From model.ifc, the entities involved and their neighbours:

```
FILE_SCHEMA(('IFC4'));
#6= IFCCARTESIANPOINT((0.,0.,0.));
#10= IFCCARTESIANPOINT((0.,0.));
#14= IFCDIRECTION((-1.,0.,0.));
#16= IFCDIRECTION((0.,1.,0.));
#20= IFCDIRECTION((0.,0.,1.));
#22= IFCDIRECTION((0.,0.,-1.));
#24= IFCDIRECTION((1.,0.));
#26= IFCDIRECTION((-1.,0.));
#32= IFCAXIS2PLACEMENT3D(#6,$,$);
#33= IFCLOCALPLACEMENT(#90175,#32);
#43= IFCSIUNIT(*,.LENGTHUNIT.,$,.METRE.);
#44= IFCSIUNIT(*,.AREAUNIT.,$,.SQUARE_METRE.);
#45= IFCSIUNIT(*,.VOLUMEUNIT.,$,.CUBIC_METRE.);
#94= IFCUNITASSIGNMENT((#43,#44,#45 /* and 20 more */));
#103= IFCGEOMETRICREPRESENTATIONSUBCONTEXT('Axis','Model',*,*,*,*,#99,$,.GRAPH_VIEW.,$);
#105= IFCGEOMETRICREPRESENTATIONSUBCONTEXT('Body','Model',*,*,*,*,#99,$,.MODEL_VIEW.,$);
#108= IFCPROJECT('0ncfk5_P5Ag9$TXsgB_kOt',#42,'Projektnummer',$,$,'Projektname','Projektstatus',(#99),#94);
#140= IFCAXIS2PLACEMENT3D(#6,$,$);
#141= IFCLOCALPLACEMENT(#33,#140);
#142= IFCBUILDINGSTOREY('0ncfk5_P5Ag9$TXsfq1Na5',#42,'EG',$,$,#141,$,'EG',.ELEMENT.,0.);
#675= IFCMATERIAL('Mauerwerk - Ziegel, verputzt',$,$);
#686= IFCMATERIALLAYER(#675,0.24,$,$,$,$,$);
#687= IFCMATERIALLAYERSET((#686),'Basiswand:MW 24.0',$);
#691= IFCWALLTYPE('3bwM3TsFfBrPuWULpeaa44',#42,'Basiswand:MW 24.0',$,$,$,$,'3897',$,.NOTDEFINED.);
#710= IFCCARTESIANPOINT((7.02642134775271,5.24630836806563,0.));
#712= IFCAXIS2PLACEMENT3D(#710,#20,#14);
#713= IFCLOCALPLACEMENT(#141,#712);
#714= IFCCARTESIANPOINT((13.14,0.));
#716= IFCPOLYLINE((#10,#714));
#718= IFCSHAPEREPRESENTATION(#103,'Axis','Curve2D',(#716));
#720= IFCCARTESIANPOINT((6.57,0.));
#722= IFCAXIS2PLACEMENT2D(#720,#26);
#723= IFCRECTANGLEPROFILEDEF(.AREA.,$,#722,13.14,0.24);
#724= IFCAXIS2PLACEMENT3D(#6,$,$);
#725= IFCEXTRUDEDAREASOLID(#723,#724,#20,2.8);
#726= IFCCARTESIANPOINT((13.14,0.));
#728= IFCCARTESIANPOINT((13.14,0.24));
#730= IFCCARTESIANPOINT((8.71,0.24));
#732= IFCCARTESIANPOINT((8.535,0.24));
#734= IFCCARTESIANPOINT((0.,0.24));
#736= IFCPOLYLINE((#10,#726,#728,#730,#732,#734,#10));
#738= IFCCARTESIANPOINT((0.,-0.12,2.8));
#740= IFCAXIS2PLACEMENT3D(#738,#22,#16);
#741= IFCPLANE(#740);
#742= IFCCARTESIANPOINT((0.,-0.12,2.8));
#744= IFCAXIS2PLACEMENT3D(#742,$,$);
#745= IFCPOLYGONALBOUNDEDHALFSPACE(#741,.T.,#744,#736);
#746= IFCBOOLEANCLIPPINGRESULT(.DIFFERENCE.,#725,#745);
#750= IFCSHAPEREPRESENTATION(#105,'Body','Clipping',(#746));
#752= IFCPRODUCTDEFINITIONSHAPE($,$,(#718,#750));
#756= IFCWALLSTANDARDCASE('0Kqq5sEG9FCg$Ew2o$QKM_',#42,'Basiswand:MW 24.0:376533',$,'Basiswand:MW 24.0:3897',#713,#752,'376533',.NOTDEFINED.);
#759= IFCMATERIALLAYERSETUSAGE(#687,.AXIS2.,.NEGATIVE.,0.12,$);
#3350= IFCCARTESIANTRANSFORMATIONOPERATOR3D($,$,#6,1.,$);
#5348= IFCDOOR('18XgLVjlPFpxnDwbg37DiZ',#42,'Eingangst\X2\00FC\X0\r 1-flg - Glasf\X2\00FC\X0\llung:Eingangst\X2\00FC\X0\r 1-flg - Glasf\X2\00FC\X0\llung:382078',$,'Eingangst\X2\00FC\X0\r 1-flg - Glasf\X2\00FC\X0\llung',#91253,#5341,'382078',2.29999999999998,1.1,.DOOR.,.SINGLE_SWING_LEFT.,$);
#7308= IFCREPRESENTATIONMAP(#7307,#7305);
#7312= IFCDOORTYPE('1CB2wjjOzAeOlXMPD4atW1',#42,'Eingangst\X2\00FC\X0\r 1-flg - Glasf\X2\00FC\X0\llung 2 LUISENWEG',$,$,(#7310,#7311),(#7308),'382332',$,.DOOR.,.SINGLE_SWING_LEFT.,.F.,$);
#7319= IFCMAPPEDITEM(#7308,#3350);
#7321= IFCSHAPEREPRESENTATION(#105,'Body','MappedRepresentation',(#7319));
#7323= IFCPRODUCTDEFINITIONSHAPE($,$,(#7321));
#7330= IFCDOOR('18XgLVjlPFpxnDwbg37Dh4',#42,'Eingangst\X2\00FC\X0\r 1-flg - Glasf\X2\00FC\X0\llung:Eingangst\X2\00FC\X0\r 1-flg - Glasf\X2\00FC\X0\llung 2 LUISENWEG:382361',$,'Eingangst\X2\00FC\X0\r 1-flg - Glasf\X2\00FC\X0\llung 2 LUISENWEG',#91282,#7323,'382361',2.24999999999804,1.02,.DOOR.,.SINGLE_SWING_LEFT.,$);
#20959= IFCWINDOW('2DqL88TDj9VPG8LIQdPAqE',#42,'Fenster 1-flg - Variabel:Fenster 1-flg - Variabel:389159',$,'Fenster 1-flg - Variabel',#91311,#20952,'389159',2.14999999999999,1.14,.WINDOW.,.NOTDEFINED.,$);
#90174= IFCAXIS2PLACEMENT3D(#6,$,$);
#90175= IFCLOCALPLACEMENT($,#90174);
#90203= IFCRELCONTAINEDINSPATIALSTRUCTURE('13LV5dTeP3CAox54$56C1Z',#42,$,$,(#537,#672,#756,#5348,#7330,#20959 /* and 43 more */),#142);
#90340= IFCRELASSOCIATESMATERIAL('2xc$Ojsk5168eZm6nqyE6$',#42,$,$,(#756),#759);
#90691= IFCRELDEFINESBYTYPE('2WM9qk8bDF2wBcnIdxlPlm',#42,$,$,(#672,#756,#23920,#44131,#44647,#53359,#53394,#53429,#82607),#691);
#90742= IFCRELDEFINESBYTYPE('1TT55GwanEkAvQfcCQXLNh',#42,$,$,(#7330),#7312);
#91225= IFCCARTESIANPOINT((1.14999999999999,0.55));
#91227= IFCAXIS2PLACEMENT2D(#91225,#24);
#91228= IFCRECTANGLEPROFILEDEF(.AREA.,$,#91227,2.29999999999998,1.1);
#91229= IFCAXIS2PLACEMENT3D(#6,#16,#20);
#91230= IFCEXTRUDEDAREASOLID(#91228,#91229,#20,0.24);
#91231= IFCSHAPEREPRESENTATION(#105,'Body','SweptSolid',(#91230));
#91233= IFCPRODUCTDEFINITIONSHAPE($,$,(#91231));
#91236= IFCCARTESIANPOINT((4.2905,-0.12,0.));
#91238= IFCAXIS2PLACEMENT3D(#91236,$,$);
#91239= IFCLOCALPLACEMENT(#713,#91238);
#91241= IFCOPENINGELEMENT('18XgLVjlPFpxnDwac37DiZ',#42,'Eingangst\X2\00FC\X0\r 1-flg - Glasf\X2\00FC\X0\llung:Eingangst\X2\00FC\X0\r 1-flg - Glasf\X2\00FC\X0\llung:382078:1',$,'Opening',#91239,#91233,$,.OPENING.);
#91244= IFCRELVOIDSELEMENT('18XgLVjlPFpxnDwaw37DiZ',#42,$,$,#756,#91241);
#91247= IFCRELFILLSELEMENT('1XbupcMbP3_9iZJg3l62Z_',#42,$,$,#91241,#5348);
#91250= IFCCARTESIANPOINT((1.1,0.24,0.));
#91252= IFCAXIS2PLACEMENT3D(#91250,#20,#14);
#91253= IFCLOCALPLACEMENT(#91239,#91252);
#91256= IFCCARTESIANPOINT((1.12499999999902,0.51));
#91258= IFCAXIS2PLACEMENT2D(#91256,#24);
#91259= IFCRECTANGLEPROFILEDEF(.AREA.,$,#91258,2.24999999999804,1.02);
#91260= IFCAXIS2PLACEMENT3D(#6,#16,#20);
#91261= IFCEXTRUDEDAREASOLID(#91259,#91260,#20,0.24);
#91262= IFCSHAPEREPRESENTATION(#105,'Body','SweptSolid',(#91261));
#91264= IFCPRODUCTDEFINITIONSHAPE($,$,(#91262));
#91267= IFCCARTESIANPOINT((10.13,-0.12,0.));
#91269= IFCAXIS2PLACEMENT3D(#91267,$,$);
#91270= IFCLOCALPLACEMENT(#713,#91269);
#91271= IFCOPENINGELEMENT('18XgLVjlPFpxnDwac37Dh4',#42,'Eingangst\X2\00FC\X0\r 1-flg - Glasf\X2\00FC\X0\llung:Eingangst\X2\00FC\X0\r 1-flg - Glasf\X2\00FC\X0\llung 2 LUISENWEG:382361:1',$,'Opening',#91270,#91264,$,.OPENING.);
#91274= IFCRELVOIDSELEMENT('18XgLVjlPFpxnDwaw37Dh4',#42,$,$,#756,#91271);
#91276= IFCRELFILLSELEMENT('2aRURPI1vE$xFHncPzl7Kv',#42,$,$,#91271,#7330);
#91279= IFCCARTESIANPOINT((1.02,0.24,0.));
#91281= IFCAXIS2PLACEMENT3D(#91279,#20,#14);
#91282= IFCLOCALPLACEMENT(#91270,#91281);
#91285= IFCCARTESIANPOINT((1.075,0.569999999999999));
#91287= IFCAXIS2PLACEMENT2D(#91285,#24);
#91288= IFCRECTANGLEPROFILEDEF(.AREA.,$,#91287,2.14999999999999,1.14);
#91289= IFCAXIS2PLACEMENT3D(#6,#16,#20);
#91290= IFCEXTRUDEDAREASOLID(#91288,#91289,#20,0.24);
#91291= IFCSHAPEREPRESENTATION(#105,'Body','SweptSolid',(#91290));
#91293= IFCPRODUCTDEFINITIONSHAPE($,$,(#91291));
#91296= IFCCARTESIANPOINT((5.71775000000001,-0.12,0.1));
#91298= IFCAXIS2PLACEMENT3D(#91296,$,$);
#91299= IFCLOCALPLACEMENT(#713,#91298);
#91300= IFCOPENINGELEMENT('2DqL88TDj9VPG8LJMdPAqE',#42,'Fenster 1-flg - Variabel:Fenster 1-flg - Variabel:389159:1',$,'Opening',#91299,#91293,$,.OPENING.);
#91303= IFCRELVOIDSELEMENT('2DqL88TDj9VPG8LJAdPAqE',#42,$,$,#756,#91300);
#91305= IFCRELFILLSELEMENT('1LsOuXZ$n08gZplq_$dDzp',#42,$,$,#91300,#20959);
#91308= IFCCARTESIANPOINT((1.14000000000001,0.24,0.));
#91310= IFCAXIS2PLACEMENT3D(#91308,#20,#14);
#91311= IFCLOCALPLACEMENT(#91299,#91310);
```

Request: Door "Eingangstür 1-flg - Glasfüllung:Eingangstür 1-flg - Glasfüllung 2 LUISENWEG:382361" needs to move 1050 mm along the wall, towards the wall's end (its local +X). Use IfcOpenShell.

```python
import ifcopenshell
import ifcopenshell.api.geometry
import ifcopenshell.util.placement

model = ifcopenshell.open("model.ifc")

door = model.by_guid("18XgLVjlPFpxnDwbg37Dh4")
opening = door.FillsVoids[0].RelatingOpeningElement
wall = opening.VoidsElements[0].RelatingBuildingElement

wall_matrix = ifcopenshell.util.placement.get_local_placement(wall.ObjectPlacement)
shift = wall_matrix[:3, 0] * 1.05
before = ifcopenshell.util.placement.get_local_placement(door.ObjectPlacement)[:3, 3].copy()

# The door is placed relative to its opening, so it follows when the opening moves.
matrix = ifcopenshell.util.placement.get_local_placement(opening.ObjectPlacement)
matrix[:3, 3] += shift
ifcopenshell.api.geometry.edit_object_placement(
    model, product=opening, matrix=matrix, is_si=False, should_transform_children=True
)

after = ifcopenshell.util.placement.get_local_placement(door.ObjectPlacement)[:3, 3]
print("door moved by", (after - before).round(3) + 0.0)

model.write("model_v2.ifc")
```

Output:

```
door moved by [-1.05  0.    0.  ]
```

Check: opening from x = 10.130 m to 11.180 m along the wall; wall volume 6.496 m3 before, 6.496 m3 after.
